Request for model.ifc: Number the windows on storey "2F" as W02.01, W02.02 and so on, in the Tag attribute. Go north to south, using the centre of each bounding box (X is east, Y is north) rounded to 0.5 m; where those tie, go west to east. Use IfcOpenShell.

First a look at what the model holds.

```python
import ifcopenshell
import ifcopenshell.util.element
import ifcopenshell.util.placement

model = ifcopenshell.open("model.ifc")
print(model.schema)
storey = next(s for s in model.by_type("IfcBuildingStorey") if s.Name == "2F")
windows = [e for e in ifcopenshell.util.element.get_decomposition(storey) if e.is_a("IfcWindow")]
for e in sorted(windows, key=lambda e: e.id()):
    origin = ifcopenshell.util.placement.get_local_placement(e.ObjectPlacement)[:3, 3]
    print(e.id(), e.Tag, e.Name, origin.round(2) + 0.0, sep=" | ")
```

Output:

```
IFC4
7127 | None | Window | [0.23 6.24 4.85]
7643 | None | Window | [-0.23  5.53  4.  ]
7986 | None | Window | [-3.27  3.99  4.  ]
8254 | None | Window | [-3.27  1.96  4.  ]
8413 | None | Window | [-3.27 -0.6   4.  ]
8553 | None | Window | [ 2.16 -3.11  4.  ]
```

```python
import ifcopenshell
import ifcopenshell.geom
import ifcopenshell.util.element
import ifcopenshell.util.shape

model = ifcopenshell.open("model.ifc")
settings = ifcopenshell.geom.settings()
settings.set("use-world-coords", True)


def centre(element):
    shape = ifcopenshell.geom.create_shape(settings, element)
    return ifcopenshell.util.shape.get_bbox_centroid(shape.geometry)


storey = next(s for s in model.by_type("IfcBuildingStorey") if s.Name == "2F")
windows = [e for e in ifcopenshell.util.element.get_decomposition(storey) if e.is_a("IfcWindow")]

# Insertion points can sit at a corner or the storey origin, so sort by the geometry (in metres).
centres = {e: centre(e) for e in windows}
windows.sort(key=lambda e: (-round(centres[e][1] / 0.5), centres[e][0]))

for i, e in enumerate(windows, start=1):
    number = f"W02.{i:02d}"
    e.Tag = number
    print(e.id(), number)

model.write("model_updated.ifc")
```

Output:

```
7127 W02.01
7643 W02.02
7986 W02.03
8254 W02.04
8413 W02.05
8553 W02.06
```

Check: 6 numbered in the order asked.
